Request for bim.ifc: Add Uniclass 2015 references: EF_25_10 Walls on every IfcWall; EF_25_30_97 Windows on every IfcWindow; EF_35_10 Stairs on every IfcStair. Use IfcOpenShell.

First a look at what the model holds.

```python
import ifcopenshell

model = ifcopenshell.open("bim.ifc")
print(model.schema)
print("classifications:", [c.Name for c in model.by_type("IfcClassification")])
for ifc_class in ("IfcDoor", "IfcRoof", "IfcStair", "IfcWall", "IfcWindow"):
    print(ifc_class, len(model.by_type(ifc_class)))
```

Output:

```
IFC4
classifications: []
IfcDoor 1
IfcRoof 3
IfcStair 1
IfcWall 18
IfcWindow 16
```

```python
import ifcopenshell
import ifcopenshell.api.classification

model = ifcopenshell.open("bim.ifc")

system = ifcopenshell.api.classification.add_classification(model, classification="Uniclass 2015")

codes = {
    "IfcWall": ("EF_25_10", "Walls"),
    "IfcWindow": ("EF_25_30_97", "Windows"),
    "IfcStair": ("EF_35_10", "Stairs"),
}
for ifc_class, (code, name) in codes.items():
    products = model.by_type(ifc_class)
    ifcopenshell.api.classification.add_reference(
        model, products=products, classification=system, identification=code, name=name
    )
    print(code, len(products))

model.write("bim_rev.ifc")
```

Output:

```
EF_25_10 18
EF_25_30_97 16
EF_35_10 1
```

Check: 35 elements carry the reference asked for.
